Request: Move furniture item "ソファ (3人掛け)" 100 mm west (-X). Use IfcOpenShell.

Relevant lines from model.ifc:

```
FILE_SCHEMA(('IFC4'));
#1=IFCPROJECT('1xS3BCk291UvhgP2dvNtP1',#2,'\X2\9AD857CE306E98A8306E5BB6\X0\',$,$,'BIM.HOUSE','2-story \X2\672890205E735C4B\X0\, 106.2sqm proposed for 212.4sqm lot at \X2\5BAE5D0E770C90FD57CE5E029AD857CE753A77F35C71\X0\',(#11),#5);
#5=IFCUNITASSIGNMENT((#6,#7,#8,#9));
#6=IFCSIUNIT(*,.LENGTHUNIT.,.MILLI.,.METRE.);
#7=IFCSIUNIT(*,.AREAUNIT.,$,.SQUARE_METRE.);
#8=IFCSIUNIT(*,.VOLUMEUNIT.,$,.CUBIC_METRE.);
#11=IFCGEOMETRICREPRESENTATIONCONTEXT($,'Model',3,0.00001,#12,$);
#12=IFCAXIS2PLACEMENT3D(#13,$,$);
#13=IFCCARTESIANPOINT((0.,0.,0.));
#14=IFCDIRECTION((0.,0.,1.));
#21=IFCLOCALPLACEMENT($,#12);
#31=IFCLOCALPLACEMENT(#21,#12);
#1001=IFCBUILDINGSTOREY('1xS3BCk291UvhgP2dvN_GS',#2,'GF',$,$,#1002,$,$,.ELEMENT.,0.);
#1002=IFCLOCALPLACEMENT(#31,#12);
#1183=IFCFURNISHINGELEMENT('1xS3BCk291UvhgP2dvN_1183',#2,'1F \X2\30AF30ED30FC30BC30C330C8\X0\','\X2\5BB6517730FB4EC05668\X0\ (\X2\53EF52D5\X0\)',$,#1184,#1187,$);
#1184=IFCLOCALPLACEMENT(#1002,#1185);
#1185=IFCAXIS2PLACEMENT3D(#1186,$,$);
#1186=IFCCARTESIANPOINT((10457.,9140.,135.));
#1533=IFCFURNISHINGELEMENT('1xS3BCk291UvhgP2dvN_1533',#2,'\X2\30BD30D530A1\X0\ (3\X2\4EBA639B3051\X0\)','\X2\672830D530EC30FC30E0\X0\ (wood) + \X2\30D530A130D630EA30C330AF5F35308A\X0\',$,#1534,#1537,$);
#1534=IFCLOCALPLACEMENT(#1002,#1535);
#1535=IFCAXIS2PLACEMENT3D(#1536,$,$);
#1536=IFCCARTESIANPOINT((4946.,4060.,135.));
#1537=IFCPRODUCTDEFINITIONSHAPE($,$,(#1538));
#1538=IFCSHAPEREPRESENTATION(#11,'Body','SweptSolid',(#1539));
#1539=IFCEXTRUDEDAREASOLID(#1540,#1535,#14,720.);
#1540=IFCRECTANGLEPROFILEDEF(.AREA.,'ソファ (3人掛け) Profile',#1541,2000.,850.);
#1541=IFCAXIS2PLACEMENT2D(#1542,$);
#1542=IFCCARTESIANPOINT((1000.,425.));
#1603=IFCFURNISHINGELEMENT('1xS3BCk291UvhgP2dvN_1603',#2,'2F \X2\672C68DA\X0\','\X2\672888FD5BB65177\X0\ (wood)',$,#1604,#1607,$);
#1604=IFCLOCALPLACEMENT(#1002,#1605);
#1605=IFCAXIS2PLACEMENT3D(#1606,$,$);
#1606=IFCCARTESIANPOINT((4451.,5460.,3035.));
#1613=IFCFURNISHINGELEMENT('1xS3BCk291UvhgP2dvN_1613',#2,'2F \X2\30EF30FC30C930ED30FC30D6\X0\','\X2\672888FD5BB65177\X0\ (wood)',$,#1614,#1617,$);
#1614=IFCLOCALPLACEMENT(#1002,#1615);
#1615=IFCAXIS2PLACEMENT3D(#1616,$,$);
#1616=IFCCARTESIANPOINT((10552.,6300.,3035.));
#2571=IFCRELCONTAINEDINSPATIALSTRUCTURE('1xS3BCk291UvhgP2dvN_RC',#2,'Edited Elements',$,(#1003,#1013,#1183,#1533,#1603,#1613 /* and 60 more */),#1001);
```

```python
import ifcopenshell
import ifcopenshell.api.geometry
import ifcopenshell.util.placement
import ifcopenshell.util.unit

model = ifcopenshell.open("model.ifc")
unit_scale = ifcopenshell.util.unit.calculate_unit_scale(model)

item = model.by_guid("1xS3BCk291UvhgP2dvN_1533")
matrix = ifcopenshell.util.placement.get_local_placement(item.ObjectPlacement)
matrix[0, 3] -= 0.1 / unit_scale
ifcopenshell.api.geometry.edit_object_placement(model, product=item, matrix=matrix, is_si=False)

print(ifcopenshell.util.placement.get_local_placement(item.ObjectPlacement).round(3) + 0.0)

model.write("model_rev.ifc")
```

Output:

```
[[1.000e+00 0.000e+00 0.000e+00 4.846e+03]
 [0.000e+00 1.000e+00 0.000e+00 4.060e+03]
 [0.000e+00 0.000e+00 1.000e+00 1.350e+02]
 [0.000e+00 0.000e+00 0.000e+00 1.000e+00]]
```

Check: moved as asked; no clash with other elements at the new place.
